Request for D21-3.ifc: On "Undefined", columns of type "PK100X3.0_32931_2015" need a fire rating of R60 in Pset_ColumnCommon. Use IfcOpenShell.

First a look at what the model holds.

```python
import ifcopenshell
import ifcopenshell.util.element

model = ifcopenshell.open("D21-3.ifc")
print(model.schema)
storey = next(s for s in model.by_type("IfcBuildingStorey") if s.Name == "Undefined")
columns = [e for e in ifcopenshell.util.element.get_decomposition(storey) if e.is_a("IfcColumn")]
seen = {}
for e in columns:
    element_type = ifcopenshell.util.element.get_type(e)
    key = (element_type.Name if element_type != e and element_type else None, ifcopenshell.util.element.get_pset(e, "Pset_ColumnCommon", "FireRating"))
    seen[key] = seen.get(key, 0) + 1
for (name, value), count in sorted(seen.items(), key=str):
    print(count, "x", name, "|", value)
```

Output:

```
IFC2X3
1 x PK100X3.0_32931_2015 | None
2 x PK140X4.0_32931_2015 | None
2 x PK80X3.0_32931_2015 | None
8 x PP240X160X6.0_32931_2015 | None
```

```python
import ifcopenshell
import ifcopenshell.api.pset
import ifcopenshell.util.element

model = ifcopenshell.open("D21-3.ifc")

storey = next(s for s in model.by_type("IfcBuildingStorey") if s.Name == "Undefined")
columns = [e for e in ifcopenshell.util.element.get_decomposition(storey) if e.is_a("IfcColumn")]

count = 0
for e in columns:
    element_type = ifcopenshell.util.element.get_type(e)
    if element_type in (None, e) or element_type.Name != "PK100X3.0_32931_2015":
        continue
    # add_pset returns the element's existing set when there is one.
    pset = ifcopenshell.api.pset.add_pset(model, product=e, name="Pset_ColumnCommon")
    ifcopenshell.api.pset.edit_pset(model, pset=pset, properties={"FireRating": "R60"})
    count += 1

print(count, "columns updated")

model.write("D21-3_v2.ifc")
```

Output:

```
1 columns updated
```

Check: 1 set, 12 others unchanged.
